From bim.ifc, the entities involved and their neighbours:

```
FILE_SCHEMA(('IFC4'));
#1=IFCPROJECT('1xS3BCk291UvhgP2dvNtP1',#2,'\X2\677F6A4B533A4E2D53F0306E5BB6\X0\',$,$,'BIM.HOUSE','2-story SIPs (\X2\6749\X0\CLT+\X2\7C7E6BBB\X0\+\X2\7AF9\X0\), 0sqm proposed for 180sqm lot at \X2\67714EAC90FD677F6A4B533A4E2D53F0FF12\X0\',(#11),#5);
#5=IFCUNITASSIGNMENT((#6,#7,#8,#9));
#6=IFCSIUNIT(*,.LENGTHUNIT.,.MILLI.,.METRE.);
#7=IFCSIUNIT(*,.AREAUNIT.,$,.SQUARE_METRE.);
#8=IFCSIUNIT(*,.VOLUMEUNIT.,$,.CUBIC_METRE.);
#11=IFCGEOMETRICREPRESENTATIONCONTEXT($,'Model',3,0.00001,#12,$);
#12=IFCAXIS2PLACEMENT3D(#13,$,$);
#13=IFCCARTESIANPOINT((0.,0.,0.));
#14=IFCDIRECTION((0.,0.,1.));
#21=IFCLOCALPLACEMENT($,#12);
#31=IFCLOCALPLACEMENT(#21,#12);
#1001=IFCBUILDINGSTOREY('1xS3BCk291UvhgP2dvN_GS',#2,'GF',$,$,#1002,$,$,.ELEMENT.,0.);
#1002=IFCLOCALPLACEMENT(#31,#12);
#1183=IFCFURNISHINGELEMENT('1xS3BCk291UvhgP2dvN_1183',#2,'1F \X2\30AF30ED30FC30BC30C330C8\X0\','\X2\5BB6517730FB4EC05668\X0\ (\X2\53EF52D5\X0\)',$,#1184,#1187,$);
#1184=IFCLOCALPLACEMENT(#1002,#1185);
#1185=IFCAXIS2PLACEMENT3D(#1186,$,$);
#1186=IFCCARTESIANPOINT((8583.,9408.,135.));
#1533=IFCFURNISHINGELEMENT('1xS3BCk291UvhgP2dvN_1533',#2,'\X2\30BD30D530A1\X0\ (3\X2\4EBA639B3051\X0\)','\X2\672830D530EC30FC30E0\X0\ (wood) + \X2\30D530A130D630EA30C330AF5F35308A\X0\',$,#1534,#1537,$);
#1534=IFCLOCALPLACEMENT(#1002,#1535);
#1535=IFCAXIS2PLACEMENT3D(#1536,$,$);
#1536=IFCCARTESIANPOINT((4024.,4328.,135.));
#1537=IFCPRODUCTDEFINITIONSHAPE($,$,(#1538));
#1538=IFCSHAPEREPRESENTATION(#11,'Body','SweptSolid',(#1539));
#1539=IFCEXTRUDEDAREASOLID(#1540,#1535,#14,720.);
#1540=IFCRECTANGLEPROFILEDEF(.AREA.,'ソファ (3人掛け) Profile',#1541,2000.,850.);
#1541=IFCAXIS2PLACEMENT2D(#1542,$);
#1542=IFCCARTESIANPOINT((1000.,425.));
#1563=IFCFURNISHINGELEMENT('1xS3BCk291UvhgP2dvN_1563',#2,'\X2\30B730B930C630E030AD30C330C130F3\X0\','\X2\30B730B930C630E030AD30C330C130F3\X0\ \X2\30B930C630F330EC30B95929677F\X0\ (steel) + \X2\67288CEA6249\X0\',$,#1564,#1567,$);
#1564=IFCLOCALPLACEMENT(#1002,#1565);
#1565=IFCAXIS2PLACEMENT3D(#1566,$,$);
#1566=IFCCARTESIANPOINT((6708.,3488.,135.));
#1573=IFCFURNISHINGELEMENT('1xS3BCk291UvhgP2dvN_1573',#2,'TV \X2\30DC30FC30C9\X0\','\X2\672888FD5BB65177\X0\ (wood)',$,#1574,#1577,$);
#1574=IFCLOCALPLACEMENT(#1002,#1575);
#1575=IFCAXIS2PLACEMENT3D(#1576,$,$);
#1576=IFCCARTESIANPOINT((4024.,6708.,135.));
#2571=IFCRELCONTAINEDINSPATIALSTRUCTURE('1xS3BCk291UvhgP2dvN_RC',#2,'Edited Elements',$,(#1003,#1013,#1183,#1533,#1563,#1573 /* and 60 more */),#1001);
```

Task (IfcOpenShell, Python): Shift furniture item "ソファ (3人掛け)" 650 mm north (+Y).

```python
import ifcopenshell
import ifcopenshell.api.geometry
import ifcopenshell.util.placement
import ifcopenshell.util.unit

model = ifcopenshell.open("bim.ifc")
unit_scale = ifcopenshell.util.unit.calculate_unit_scale(model)

item = model.by_guid("1xS3BCk291UvhgP2dvN_1533")
matrix = ifcopenshell.util.placement.get_local_placement(item.ObjectPlacement)
matrix[1, 3] += 0.65 / unit_scale
ifcopenshell.api.geometry.edit_object_placement(model, product=item, matrix=matrix, is_si=False)

print(ifcopenshell.util.placement.get_local_placement(item.ObjectPlacement).round(3) + 0.0)

model.write("bim_updated.ifc")
```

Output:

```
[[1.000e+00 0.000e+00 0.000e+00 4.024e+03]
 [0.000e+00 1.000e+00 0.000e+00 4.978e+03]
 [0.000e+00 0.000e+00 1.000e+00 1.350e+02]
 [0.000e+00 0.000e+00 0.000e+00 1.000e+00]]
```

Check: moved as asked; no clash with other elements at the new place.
